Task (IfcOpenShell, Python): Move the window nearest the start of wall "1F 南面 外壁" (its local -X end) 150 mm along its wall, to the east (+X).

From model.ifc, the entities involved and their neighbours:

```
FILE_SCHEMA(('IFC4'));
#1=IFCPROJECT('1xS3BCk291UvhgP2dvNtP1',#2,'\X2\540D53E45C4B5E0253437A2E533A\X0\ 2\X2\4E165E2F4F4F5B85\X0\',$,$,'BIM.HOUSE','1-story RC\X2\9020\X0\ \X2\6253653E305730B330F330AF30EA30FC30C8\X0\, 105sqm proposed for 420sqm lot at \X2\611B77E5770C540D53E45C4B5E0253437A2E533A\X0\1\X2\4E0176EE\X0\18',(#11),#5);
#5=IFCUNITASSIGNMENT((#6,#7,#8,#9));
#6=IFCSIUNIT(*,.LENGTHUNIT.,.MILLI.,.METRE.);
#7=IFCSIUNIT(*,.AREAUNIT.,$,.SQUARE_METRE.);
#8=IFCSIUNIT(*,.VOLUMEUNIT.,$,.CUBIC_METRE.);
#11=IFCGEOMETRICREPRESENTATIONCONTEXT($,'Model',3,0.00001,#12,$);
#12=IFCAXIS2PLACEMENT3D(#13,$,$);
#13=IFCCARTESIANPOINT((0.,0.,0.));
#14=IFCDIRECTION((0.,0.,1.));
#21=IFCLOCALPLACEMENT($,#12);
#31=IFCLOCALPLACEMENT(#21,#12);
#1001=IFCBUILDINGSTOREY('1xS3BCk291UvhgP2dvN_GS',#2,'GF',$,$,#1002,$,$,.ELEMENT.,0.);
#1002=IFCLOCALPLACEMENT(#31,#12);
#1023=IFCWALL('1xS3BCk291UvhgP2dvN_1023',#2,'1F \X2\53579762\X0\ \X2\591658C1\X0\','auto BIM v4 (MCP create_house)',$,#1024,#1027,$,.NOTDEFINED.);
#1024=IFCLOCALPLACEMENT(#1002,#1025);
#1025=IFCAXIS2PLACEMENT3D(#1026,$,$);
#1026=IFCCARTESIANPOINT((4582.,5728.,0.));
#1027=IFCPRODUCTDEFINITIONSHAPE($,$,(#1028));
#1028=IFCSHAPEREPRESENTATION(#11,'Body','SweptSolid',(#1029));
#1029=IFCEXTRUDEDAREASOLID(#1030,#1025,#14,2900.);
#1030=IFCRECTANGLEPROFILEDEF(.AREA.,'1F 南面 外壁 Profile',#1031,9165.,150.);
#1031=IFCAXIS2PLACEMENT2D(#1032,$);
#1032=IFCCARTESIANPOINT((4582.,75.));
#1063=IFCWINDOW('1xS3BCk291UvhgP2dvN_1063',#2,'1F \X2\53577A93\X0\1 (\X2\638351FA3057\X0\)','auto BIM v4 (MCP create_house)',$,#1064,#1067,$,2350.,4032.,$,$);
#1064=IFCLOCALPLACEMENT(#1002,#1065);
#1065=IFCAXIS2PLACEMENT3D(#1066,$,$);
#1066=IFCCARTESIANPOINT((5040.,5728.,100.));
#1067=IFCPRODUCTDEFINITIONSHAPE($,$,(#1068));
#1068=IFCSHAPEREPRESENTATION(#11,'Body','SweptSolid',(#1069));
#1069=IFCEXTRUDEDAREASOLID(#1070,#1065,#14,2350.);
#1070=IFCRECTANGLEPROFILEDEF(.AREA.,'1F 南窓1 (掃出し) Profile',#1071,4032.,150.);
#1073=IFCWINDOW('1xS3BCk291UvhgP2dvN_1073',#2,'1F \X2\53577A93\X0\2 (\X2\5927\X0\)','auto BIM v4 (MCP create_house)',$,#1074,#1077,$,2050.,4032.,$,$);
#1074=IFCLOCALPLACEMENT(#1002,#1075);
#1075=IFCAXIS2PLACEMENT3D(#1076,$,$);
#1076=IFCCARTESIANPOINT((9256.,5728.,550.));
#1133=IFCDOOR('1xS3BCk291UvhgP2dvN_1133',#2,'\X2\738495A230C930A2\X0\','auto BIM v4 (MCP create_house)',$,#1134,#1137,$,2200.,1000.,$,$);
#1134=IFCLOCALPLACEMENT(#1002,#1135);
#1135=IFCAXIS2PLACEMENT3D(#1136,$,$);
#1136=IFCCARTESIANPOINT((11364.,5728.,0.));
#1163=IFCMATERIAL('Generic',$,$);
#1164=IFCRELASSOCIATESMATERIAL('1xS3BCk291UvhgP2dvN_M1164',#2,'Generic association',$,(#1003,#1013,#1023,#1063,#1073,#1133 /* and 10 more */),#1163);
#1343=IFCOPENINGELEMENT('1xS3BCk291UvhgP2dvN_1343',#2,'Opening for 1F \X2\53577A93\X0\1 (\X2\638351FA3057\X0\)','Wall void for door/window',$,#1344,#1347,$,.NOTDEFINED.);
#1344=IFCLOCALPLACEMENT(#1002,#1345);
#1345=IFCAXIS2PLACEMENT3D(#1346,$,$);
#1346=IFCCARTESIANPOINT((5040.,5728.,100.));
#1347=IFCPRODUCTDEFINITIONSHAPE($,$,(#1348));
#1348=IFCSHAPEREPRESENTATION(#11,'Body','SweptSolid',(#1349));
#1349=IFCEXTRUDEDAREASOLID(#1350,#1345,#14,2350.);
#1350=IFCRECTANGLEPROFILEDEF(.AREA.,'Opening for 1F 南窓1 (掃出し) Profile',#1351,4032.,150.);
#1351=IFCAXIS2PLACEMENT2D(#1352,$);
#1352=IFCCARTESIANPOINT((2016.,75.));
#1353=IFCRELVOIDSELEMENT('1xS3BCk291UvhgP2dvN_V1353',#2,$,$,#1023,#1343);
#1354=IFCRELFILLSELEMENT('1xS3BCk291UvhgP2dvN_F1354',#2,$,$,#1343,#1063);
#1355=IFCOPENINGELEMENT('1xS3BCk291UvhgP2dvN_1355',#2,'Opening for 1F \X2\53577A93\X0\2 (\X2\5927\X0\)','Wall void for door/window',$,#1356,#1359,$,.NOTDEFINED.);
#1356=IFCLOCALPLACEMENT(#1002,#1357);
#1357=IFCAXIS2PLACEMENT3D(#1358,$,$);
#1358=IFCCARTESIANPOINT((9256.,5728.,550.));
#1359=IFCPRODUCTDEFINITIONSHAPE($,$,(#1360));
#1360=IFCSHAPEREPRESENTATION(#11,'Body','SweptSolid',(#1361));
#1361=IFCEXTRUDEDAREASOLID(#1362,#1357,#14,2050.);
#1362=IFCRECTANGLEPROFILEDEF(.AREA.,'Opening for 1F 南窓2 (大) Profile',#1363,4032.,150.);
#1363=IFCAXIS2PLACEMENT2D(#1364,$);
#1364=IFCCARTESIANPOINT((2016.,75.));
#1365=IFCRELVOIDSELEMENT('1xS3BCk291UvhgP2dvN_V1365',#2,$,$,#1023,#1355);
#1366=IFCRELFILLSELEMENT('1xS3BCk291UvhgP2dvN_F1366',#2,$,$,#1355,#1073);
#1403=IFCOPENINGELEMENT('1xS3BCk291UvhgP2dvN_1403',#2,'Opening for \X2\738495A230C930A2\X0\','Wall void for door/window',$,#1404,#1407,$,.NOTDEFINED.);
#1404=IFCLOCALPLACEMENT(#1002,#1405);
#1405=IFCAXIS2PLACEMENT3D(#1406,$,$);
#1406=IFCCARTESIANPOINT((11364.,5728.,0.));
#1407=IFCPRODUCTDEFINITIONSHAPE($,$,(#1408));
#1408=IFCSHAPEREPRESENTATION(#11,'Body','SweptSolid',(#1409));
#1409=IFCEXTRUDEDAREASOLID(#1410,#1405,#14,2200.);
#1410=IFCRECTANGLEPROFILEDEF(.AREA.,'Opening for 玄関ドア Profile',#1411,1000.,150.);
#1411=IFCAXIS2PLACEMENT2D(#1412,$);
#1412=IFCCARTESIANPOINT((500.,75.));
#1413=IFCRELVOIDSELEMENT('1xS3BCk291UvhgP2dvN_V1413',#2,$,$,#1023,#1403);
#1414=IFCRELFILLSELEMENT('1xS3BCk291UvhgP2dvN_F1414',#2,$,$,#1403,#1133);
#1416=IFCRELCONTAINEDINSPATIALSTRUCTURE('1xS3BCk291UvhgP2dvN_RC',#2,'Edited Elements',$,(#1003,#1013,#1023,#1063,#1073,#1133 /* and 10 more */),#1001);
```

```python
import ifcopenshell
import ifcopenshell.api.geometry
import ifcopenshell.util.placement
import ifcopenshell.util.unit

model = ifcopenshell.open("model.ifc")
unit_scale = ifcopenshell.util.unit.calculate_unit_scale(model)

window = model.by_guid("1xS3BCk291UvhgP2dvN_1063")
opening = window.FillsVoids[0].RelatingOpeningElement
wall = opening.VoidsElements[0].RelatingBuildingElement

wall_matrix = ifcopenshell.util.placement.get_local_placement(wall.ObjectPlacement)
shift = wall_matrix[:3, 0] * 0.15 / unit_scale
before = ifcopenshell.util.placement.get_local_placement(window.ObjectPlacement)[:3, 3].copy()

# The window is not placed relative to its opening, so move both.
for product in (opening, window):
    matrix = ifcopenshell.util.placement.get_local_placement(product.ObjectPlacement)
    matrix[:3, 3] += shift
    ifcopenshell.api.geometry.edit_object_placement(model, product=product, matrix=matrix, is_si=False)

after = ifcopenshell.util.placement.get_local_placement(window.ObjectPlacement)[:3, 3]
print("window moved by", (after - before).round(3) + 0.0)

model.write("model-out.ifc")
```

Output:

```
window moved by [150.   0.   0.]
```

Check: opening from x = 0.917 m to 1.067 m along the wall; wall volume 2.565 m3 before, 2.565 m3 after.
